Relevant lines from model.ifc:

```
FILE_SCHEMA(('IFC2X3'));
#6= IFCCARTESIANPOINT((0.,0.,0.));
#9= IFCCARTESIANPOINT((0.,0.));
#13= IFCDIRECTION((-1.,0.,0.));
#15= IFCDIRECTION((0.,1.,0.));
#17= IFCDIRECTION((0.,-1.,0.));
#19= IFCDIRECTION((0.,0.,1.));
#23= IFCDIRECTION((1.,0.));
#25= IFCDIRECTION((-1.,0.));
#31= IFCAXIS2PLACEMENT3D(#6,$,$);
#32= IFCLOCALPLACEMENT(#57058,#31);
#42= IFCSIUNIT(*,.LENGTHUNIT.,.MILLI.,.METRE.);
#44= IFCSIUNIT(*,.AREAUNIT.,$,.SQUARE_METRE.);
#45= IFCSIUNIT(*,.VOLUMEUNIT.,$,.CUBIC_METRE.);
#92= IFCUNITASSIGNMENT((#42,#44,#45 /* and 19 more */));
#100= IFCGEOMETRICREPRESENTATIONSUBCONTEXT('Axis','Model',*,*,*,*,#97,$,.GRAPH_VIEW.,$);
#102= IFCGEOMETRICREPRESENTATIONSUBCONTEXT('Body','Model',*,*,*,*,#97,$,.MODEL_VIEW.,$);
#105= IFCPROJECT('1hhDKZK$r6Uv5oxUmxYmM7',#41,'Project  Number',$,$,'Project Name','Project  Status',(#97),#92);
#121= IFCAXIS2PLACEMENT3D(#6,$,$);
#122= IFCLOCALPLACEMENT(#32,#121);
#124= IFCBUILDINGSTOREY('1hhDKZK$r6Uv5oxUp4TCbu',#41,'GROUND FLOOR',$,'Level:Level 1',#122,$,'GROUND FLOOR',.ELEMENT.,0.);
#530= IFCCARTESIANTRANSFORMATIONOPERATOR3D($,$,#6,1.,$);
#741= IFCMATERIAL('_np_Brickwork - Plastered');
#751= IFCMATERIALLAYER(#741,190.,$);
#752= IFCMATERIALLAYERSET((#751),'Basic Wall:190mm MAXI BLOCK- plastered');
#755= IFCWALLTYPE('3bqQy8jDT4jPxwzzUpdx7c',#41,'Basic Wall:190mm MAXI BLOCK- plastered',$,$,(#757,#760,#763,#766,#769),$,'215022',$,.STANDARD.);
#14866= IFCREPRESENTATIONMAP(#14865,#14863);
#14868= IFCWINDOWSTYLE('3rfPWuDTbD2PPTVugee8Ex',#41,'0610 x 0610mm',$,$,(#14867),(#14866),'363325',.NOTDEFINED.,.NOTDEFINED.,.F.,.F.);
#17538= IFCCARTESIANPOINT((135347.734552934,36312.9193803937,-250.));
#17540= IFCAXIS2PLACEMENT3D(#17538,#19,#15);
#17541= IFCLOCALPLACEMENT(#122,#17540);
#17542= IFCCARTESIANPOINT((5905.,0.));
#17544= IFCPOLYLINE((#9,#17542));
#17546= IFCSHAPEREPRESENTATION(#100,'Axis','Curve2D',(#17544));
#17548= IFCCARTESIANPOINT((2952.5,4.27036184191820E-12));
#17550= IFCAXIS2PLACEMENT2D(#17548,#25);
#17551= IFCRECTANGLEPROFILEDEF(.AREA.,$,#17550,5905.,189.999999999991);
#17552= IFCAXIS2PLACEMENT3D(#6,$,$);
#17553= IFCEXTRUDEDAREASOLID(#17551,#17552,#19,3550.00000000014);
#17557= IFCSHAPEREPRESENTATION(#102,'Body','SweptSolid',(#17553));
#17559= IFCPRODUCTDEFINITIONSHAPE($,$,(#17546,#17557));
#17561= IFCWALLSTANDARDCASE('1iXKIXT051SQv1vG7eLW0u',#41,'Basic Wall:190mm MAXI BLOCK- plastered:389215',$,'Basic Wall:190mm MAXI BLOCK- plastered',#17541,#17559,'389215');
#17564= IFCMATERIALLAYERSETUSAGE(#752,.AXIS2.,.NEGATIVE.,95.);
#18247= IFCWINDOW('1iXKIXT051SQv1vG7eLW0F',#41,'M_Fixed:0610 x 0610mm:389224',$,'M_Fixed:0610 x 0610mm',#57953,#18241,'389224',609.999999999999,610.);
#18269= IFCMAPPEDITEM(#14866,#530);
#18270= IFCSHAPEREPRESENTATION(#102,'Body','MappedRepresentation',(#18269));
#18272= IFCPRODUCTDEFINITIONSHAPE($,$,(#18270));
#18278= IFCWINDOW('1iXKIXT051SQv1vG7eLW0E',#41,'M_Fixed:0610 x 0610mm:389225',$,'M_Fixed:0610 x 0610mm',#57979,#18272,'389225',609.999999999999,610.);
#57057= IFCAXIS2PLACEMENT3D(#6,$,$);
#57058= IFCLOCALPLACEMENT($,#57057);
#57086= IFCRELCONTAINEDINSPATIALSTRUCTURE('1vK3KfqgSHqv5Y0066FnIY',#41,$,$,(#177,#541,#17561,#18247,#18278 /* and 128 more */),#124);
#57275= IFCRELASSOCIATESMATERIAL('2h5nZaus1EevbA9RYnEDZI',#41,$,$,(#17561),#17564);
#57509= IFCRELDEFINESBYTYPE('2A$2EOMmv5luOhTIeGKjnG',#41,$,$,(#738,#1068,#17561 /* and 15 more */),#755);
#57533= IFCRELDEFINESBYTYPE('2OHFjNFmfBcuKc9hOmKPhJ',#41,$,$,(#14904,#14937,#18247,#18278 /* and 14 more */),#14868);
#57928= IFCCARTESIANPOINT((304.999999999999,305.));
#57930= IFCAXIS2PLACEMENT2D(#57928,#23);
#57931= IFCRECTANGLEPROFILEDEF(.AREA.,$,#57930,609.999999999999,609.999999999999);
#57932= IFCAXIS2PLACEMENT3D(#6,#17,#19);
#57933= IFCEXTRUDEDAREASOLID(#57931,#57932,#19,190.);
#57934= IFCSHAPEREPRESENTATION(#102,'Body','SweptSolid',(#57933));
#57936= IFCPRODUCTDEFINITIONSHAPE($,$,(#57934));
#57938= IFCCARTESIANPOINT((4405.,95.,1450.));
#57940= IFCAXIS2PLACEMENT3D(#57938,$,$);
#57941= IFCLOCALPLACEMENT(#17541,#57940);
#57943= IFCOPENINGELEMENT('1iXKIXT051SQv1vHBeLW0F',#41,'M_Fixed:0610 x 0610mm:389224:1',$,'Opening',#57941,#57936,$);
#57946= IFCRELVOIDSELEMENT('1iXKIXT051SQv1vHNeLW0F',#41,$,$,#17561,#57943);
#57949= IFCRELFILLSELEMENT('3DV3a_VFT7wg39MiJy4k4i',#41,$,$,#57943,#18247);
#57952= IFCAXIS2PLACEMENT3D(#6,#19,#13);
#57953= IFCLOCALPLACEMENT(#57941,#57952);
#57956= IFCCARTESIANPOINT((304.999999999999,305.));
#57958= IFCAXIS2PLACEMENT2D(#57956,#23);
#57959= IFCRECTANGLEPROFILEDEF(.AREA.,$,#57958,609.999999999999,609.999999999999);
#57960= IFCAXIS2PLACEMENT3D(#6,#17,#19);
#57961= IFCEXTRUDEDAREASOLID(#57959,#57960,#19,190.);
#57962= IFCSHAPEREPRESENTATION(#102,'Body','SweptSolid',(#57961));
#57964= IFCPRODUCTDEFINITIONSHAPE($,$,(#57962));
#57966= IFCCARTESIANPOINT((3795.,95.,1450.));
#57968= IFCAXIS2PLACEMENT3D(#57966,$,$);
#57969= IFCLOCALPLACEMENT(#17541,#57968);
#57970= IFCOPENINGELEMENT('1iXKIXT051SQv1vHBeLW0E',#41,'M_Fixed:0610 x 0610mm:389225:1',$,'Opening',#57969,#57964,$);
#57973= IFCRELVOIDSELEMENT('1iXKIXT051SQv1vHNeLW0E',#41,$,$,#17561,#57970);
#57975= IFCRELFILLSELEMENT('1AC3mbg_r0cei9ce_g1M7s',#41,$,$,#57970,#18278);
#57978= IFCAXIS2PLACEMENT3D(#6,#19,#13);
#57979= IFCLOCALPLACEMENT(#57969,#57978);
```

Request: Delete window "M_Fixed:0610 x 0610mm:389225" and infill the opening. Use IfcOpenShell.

```python
import ifcopenshell
import ifcopenshell.api.feature
import ifcopenshell.api.root
import ifcopenshell.geom
import ifcopenshell.util.shape

model = ifcopenshell.open("model.ifc")
settings = ifcopenshell.geom.settings()


def volume(element):
    """Net volume in cubic metres, openings subtracted."""
    shape = ifcopenshell.geom.create_shape(settings, element)
    return ifcopenshell.util.shape.get_volume(shape.geometry)


window = model.by_guid("1iXKIXT051SQv1vG7eLW0E")
opening = window.FillsVoids[0].RelatingOpeningElement
wall = opening.VoidsElements[0].RelatingBuildingElement
before = volume(wall)

ifcopenshell.api.root.remove_product(model, product=window)
ifcopenshell.api.feature.remove_feature(model, feature=opening)

after = volume(wall)

print(f"wall volume {before:.3f} -> {after:.3f} m3")

model.write("model_edited.ifc")
```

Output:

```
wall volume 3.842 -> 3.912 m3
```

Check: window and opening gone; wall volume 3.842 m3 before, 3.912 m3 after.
